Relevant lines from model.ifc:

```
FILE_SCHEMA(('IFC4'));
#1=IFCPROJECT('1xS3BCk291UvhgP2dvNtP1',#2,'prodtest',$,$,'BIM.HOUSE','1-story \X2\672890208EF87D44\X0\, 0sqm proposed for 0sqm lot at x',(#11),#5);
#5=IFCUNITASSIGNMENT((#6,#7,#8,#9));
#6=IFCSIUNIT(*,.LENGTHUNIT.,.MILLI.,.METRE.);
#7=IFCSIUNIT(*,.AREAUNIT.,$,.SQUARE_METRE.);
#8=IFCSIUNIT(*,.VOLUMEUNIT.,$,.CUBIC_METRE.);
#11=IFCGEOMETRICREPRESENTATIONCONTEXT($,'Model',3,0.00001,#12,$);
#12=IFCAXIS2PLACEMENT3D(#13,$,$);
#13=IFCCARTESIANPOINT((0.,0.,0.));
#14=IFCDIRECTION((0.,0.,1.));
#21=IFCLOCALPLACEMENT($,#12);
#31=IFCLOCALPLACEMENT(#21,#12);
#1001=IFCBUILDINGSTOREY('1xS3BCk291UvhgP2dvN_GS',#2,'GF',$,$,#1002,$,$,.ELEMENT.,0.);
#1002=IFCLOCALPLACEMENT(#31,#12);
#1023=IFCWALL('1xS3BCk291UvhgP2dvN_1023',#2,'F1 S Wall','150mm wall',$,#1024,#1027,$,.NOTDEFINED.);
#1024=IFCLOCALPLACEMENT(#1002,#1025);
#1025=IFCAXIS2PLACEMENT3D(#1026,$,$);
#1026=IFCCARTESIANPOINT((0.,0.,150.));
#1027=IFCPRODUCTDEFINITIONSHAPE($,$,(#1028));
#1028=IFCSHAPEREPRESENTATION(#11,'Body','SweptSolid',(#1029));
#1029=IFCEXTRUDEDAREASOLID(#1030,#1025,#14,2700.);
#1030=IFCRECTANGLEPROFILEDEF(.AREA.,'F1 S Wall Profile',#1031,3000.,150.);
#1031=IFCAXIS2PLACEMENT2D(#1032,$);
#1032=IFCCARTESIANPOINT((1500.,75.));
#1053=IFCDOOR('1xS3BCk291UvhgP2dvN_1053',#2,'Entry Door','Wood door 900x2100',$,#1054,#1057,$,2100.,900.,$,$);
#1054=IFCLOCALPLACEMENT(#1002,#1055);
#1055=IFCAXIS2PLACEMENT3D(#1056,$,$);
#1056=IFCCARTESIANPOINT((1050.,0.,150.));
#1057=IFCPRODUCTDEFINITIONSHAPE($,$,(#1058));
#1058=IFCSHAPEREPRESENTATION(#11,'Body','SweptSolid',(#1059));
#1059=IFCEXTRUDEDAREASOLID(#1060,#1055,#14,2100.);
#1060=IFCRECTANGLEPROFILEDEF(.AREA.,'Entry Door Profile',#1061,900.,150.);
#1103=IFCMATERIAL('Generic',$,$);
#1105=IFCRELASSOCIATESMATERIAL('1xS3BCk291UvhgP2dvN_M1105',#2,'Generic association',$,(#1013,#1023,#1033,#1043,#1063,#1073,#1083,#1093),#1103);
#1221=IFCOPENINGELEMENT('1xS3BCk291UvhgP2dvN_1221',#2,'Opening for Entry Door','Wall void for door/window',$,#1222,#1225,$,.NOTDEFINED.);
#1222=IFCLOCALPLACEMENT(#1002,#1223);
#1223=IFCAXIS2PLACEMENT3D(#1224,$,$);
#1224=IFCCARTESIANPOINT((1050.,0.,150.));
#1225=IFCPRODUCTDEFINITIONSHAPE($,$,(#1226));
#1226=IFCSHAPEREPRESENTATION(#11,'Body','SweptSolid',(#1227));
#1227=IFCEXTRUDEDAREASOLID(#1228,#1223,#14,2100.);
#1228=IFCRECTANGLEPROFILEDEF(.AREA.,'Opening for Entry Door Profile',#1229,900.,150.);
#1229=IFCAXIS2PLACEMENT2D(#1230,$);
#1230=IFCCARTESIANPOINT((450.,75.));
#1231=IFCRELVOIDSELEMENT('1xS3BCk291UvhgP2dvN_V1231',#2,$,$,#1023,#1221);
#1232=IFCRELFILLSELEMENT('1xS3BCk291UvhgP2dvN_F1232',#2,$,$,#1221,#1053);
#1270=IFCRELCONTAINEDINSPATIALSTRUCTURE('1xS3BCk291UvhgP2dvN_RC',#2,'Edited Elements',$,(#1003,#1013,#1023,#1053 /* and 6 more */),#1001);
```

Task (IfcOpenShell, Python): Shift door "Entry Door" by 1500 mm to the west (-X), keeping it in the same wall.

```python
import ifcopenshell
import ifcopenshell.api.geometry
import ifcopenshell.util.placement
import ifcopenshell.util.unit

model = ifcopenshell.open("model.ifc")
unit_scale = ifcopenshell.util.unit.calculate_unit_scale(model)

door = model.by_guid("1xS3BCk291UvhgP2dvN_1053")
opening = door.FillsVoids[0].RelatingOpeningElement
wall = opening.VoidsElements[0].RelatingBuildingElement

wall_matrix = ifcopenshell.util.placement.get_local_placement(wall.ObjectPlacement)
shift = wall_matrix[:3, 0] * -1.5 / unit_scale
before = ifcopenshell.util.placement.get_local_placement(door.ObjectPlacement)[:3, 3].copy()

# The door is not placed relative to its opening, so move both.
for product in (opening, door):
    matrix = ifcopenshell.util.placement.get_local_placement(product.ObjectPlacement)
    matrix[:3, 3] += shift
    ifcopenshell.api.geometry.edit_object_placement(model, product=product, matrix=matrix, is_si=False)

after = ifcopenshell.util.placement.get_local_placement(door.ObjectPlacement)[:3, 3]
print("door moved by", (after - before).round(3) + 0.0)

model.write("model_v2.ifc")
```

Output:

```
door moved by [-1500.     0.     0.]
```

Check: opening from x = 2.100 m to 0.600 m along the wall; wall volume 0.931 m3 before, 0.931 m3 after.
